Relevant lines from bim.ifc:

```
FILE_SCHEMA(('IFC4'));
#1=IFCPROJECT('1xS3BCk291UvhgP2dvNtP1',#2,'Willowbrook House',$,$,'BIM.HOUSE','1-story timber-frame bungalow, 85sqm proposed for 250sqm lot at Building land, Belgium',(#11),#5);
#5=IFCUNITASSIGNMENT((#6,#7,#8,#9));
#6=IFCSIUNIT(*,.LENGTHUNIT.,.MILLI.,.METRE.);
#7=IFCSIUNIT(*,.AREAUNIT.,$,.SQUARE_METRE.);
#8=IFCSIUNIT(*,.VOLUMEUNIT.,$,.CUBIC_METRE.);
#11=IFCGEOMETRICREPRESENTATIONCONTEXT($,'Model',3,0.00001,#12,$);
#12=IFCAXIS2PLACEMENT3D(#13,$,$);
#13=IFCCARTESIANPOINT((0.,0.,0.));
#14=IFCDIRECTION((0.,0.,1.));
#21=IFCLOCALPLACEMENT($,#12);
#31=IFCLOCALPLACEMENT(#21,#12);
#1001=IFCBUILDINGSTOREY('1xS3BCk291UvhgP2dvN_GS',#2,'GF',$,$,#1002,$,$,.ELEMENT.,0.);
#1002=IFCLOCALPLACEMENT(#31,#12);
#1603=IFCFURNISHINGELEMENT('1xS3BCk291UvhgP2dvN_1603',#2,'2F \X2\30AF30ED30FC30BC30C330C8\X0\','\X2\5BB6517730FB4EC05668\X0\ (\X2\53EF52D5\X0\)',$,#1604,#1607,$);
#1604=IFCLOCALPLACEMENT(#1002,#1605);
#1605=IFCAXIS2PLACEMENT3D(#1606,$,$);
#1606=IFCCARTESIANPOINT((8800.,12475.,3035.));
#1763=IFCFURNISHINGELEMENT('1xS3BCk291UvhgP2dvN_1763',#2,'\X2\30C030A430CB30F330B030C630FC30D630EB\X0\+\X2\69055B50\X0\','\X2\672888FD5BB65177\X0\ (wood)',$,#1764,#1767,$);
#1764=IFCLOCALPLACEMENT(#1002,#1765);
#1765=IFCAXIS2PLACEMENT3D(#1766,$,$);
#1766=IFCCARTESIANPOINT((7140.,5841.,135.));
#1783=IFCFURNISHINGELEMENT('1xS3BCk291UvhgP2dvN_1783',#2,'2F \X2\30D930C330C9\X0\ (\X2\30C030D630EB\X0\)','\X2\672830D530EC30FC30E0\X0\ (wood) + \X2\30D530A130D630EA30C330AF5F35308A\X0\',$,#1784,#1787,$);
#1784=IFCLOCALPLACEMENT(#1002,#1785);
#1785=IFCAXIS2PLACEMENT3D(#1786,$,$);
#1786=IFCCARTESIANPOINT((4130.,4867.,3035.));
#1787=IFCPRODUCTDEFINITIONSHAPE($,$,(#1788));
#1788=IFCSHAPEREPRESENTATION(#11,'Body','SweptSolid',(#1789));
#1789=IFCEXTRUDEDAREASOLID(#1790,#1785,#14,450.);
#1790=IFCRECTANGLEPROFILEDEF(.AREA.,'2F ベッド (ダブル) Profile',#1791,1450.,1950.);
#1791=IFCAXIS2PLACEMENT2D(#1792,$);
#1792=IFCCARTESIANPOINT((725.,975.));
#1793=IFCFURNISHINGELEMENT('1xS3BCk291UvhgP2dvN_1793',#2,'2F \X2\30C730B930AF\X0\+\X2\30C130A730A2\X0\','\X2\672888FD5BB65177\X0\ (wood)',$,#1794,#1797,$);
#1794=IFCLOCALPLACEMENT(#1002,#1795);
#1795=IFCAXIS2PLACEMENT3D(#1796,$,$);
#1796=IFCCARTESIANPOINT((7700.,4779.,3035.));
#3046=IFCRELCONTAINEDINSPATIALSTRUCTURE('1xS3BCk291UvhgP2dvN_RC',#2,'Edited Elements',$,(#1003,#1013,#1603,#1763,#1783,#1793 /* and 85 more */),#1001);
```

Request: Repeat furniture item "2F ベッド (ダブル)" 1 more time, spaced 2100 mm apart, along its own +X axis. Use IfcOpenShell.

```python
import ifcopenshell
import ifcopenshell.api.geometry
import ifcopenshell.api.root
import ifcopenshell.util.element
import ifcopenshell.util.placement
import ifcopenshell.util.unit

model = ifcopenshell.open("bim.ifc")
unit_scale = ifcopenshell.util.unit.calculate_unit_scale(model)


def reuse_history(source, copy):
    """copy_class also copies each property set's owner history, people and application; keep the originals."""
    for rel in copy.IsDefinedBy:
        if rel.is_a("IfcRelDefinesByProperties") and (history := rel.RelatingPropertyDefinition.OwnerHistory):
            rel.RelatingPropertyDefinition.OwnerHistory = source.OwnerHistory
            ifcopenshell.util.element.remove_deep2(model, history)


source = model.by_id(1783)
base = ifcopenshell.util.placement.get_local_placement(source.ObjectPlacement)
step = base[:3, 0] * 2.1 / unit_scale

for i in range(1, 2):
    copy = ifcopenshell.api.root.copy_class(model, product=source)
    copy.Representation = ifcopenshell.util.element.copy_deep(
        model, source.Representation, exclude=["IfcGeometricRepresentationContext", "IfcRepresentationMap"]
    )
    reuse_history(source, copy)
    matrix = base.copy()
    matrix[:3, 3] += i * step
    print("added at", matrix[:3, 3].round(3) + 0.0)
    ifcopenshell.api.geometry.edit_object_placement(model, product=copy, matrix=matrix, is_si=False)

model.write("bim-out.ifc")
```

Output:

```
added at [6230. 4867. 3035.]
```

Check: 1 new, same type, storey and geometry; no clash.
